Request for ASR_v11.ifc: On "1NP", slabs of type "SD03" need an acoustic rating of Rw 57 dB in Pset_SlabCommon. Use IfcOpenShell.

First a look at what the model holds.

```python
import ifcopenshell
import ifcopenshell.util.element

model = ifcopenshell.open("ASR_v11.ifc")
print(model.schema)
storey = next(s for s in model.by_type("IfcBuildingStorey") if s.Name == "1NP")
slabs = [e for e in ifcopenshell.util.element.get_decomposition(storey) if e.is_a("IfcSlab")]
seen = {}
for e in slabs:
    element_type = ifcopenshell.util.element.get_type(e)
    key = (element_type.Name if element_type != e and element_type else None, ifcopenshell.util.element.get_pset(e, "Pset_SlabCommon", "AcousticRating"))
    seen[key] = seen.get(key, 0) + 1
for (name, value), count in sorted(seen.items(), key=str):
    print(count, "x", name, "|", value)
```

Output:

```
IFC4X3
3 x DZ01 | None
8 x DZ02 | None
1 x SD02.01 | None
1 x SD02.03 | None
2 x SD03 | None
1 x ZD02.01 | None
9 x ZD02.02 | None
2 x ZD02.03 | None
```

```python
import ifcopenshell
import ifcopenshell.api.pset
import ifcopenshell.util.element

model = ifcopenshell.open("ASR_v11.ifc")

storey = next(s for s in model.by_type("IfcBuildingStorey") if s.Name == "1NP")
slabs = [e for e in ifcopenshell.util.element.get_decomposition(storey) if e.is_a("IfcSlab")]

count = 0
for e in slabs:
    element_type = ifcopenshell.util.element.get_type(e)
    if element_type in (None, e) or element_type.Name != "SD03":
        continue
    # add_pset returns the element's existing set when there is one.
    pset = ifcopenshell.api.pset.add_pset(model, product=e, name="Pset_SlabCommon")
    ifcopenshell.api.pset.edit_pset(model, pset=pset, properties={"AcousticRating": "Rw 57 dB"})
    count += 1

print(count, "slabs updated")

model.write("ASR_v11_rev.ifc")
```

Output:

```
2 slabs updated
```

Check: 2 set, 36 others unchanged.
